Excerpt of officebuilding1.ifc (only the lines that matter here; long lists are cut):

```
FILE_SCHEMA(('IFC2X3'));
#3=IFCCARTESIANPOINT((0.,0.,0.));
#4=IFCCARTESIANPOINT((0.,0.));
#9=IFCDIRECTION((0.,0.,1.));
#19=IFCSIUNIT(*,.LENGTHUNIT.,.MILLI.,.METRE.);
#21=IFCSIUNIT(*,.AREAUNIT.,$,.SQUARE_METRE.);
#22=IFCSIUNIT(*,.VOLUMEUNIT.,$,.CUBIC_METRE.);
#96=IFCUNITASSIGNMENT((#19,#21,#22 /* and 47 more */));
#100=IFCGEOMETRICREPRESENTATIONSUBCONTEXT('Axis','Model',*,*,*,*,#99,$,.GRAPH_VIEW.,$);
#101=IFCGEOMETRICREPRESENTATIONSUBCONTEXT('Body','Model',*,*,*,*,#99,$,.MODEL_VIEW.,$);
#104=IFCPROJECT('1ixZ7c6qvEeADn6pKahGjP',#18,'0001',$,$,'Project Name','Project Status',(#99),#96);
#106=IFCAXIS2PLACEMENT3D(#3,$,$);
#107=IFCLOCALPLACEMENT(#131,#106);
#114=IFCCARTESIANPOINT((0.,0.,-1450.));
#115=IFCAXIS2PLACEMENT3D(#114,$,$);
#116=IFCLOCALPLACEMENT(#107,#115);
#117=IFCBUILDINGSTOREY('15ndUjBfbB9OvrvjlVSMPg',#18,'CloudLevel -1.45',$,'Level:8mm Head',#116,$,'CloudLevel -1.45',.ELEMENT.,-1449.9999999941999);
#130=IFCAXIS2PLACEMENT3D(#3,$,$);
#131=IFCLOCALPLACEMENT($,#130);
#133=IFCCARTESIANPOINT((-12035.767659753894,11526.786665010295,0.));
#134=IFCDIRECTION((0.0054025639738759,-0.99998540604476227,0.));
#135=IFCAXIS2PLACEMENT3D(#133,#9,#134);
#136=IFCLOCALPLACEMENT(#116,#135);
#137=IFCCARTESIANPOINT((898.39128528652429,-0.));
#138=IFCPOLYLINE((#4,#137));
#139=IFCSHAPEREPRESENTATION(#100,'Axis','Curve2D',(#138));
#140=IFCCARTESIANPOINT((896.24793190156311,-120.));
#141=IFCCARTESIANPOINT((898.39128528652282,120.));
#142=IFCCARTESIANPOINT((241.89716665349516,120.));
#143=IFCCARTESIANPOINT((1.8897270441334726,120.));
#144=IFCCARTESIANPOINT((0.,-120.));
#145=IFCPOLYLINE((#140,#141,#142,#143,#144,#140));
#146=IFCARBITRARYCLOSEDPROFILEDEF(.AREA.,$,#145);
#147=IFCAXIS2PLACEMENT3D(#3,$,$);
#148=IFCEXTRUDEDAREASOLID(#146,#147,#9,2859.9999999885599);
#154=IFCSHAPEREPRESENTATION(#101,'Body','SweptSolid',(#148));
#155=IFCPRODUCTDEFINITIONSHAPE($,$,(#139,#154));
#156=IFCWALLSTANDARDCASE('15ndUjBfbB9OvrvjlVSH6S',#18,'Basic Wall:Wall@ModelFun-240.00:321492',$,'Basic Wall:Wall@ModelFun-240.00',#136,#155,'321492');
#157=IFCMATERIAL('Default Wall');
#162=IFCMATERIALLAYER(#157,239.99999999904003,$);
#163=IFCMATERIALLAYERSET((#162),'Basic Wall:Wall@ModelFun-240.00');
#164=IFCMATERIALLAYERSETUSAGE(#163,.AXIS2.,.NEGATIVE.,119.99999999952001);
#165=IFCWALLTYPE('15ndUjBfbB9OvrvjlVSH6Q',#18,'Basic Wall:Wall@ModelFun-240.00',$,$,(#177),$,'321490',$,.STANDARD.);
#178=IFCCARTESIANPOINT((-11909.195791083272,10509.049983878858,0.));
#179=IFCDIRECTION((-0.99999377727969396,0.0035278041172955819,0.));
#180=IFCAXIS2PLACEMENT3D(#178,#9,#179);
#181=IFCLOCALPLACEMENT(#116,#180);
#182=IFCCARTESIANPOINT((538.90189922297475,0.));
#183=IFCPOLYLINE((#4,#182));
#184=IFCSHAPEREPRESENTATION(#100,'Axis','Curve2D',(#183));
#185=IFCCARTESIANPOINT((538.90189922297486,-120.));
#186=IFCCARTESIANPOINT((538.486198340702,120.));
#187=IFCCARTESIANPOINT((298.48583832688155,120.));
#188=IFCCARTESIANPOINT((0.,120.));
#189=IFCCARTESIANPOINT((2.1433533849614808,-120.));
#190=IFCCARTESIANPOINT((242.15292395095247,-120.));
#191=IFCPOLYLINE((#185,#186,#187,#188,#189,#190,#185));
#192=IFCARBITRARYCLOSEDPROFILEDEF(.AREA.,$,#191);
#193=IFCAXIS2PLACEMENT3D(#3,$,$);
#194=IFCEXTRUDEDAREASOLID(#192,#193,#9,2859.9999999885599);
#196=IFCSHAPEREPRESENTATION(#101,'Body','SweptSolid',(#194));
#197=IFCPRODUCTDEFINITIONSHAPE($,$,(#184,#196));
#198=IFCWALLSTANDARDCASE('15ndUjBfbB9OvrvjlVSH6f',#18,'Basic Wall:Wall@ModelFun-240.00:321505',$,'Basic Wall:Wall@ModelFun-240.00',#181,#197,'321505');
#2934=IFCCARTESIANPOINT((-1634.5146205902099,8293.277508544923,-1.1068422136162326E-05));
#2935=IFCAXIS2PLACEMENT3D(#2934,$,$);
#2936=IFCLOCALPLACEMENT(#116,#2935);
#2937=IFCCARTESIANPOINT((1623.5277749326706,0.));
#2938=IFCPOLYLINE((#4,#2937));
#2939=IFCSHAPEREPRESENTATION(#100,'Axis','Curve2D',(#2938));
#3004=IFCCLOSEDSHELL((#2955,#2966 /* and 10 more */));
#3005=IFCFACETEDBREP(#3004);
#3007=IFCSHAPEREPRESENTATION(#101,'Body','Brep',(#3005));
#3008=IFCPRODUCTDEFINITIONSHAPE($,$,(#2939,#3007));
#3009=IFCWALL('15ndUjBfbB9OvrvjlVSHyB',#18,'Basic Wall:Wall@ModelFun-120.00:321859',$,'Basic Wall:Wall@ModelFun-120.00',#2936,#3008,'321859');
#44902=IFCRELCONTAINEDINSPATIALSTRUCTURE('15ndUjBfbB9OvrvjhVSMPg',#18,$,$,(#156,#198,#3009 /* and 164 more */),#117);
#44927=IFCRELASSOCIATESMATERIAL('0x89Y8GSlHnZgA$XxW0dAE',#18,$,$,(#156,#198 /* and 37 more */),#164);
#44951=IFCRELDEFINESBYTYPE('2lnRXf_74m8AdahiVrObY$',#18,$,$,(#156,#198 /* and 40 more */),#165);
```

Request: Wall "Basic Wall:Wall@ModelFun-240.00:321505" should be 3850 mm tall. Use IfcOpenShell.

```python
import ifcopenshell
import ifcopenshell.geom
import ifcopenshell.util.representation
import ifcopenshell.util.shape
import ifcopenshell.util.unit

model = ifcopenshell.open("officebuilding1.ifc")
unit_scale = ifcopenshell.util.unit.calculate_unit_scale(model)
settings = ifcopenshell.geom.settings()


def volume(element):
    """Net volume in cubic metres, openings subtracted."""
    shape = ifcopenshell.geom.create_shape(settings, element)
    return ifcopenshell.util.shape.get_volume(shape.geometry)


wall = model.by_guid("15ndUjBfbB9OvrvjlVSH6f")
before = volume(wall)

body = ifcopenshell.util.representation.get_representation(wall, "Model", "Body")
solid = body.Items[0]
old_height = solid.Depth
solid.Depth = 3.85 / unit_scale
after = volume(wall)

print(f"height {old_height:g} -> {solid.Depth:g}, volume {before:.3f} -> {after:.3f} m3")

model.write("officebuilding1_updated.ifc")
```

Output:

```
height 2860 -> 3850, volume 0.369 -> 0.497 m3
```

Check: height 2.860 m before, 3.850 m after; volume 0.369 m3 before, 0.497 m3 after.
